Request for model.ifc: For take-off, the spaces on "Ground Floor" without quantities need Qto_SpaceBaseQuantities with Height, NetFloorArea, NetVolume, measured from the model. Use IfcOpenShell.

First a look at what the model holds.

```python
import ifcopenshell
import ifcopenshell.util.element
import ifcopenshell.util.unit

model = ifcopenshell.open("model.ifc")
print(model.schema)
for unit_type in ("LENGTHUNIT", "AREAUNIT", "VOLUMEUNIT"):
    print(unit_type, ifcopenshell.util.unit.calculate_unit_scale(model, unit_type))
storey = next(s for s in model.by_type("IfcBuildingStorey") if s.Name == "Ground Floor")
spaces = [e for e in ifcopenshell.util.element.get_decomposition(storey) if e.is_a("IfcSpace")]
for e in sorted(spaces, key=lambda e: e.id()):
    print(e.id(), e.is_a(), e.Name, list(ifcopenshell.util.element.get_psets(e, qtos_only=True)), sep=" | ")
```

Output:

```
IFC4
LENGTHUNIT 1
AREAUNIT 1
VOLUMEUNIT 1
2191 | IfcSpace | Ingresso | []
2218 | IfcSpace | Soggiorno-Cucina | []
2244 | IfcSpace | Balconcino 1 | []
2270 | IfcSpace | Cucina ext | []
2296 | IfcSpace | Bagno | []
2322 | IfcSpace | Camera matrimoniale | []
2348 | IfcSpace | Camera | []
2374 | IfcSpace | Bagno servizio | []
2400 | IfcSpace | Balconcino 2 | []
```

```python
import ifcopenshell
import ifcopenshell.api.pset
import ifcopenshell.geom
import ifcopenshell.util.element
import ifcopenshell.util.shape
import ifcopenshell.util.unit

model = ifcopenshell.open("model.ifc")
unit_scale = ifcopenshell.util.unit.calculate_unit_scale(model)
area_scale = ifcopenshell.util.unit.calculate_unit_scale(model, "AREAUNIT")
volume_scale = ifcopenshell.util.unit.calculate_unit_scale(model, "VOLUMEUNIT")
settings = ifcopenshell.geom.settings()

storey = next(s for s in model.by_type("IfcBuildingStorey") if s.Name == "Ground Floor")
spaces = [e for e in ifcopenshell.util.element.get_decomposition(storey) if e.is_a("IfcSpace")]

for e in sorted(spaces, key=lambda e: e.id()):
    if ifcopenshell.util.element.get_psets(e, qtos_only=True, should_inherit=False):
        continue
    # Geometry comes back in metres, in the element's own axes.
    shape = ifcopenshell.geom.create_shape(settings, e)
    values = {
        "Height": ifcopenshell.util.shape.get_z(shape.geometry) / unit_scale,
        "NetFloorArea": ifcopenshell.util.shape.get_footprint_area(shape.geometry) / area_scale,
        "NetVolume": ifcopenshell.util.shape.get_volume(shape.geometry) / volume_scale,
    }
    qto = ifcopenshell.api.pset.add_qto(model, product=e, name="Qto_SpaceBaseQuantities")
    ifcopenshell.api.pset.edit_qto(model, qto=qto, properties=values)
    print(e.id(), {k: round(v, 3) for k, v in values.items()})

model.write("model_rev.ifc")
```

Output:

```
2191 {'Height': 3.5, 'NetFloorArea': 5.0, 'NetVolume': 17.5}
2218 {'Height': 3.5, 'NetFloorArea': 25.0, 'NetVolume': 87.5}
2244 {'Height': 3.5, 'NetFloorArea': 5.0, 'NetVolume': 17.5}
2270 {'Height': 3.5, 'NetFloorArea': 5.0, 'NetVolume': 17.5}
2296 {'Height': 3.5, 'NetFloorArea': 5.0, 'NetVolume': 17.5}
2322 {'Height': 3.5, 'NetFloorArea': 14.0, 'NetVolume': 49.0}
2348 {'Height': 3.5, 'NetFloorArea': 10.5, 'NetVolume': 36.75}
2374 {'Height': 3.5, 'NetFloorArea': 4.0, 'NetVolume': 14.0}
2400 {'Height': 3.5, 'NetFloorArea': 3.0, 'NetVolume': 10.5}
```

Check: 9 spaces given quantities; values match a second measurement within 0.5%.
